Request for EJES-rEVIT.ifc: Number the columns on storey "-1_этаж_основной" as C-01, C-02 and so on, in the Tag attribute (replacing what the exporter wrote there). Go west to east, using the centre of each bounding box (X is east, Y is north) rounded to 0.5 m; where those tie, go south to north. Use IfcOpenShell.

First a look at what the model holds.

```python
import ifcopenshell
import ifcopenshell.util.element
import ifcopenshell.util.placement

model = ifcopenshell.open("EJES-rEVIT.ifc")
print(model.schema)
storey = next(s for s in model.by_type("IfcBuildingStorey") if s.Name == "-1_этаж_основной")
columns = [e for e in ifcopenshell.util.element.get_decomposition(storey) if e.is_a("IfcColumn")]
for e in sorted(columns, key=lambda e: e.id()):
    origin = ifcopenshell.util.placement.get_local_placement(e.ObjectPlacement)[:3, 3]
    print(e.id(), e.Tag, e.Name, origin.round(2) + 0.0, sep=" | ")
```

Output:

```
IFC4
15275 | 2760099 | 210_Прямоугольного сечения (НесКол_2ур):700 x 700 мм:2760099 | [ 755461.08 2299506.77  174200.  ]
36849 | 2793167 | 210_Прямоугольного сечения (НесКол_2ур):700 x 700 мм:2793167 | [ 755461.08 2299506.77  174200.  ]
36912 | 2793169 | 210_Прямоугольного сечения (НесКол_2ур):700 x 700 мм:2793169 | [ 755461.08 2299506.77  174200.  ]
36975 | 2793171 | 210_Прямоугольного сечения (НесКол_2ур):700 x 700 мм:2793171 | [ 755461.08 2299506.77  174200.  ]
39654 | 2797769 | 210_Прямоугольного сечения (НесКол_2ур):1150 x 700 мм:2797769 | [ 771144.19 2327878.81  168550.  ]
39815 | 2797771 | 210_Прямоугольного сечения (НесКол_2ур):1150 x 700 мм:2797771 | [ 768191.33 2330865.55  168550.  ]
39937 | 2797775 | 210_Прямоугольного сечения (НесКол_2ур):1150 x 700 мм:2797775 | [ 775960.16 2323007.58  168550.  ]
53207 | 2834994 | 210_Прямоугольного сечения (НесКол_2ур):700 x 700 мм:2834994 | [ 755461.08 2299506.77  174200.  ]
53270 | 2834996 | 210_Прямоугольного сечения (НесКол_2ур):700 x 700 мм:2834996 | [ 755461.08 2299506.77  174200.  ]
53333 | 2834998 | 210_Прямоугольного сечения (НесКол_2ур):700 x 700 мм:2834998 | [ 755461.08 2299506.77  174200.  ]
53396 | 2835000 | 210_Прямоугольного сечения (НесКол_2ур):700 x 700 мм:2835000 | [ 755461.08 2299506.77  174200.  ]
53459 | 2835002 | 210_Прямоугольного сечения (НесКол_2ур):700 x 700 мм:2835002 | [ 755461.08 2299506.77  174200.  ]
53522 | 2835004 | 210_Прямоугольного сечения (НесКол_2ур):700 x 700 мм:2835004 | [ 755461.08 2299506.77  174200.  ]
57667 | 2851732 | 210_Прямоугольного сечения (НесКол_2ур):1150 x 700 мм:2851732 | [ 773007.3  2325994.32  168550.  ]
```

```python
import ifcopenshell
import ifcopenshell.geom
import ifcopenshell.util.element
import ifcopenshell.util.shape

model = ifcopenshell.open("EJES-rEVIT.ifc")
settings = ifcopenshell.geom.settings()
settings.set("use-world-coords", True)


def centre(element):
    shape = ifcopenshell.geom.create_shape(settings, element)
    return ifcopenshell.util.shape.get_bbox_centroid(shape.geometry)


storey = next(s for s in model.by_type("IfcBuildingStorey") if s.Name == "-1_этаж_основной")
columns = [e for e in ifcopenshell.util.element.get_decomposition(storey) if e.is_a("IfcColumn")]

# Insertion points can sit at a corner or the storey origin, so sort by the geometry (in metres).
centres = {e: centre(e) for e in columns}
columns.sort(key=lambda e: (round(centres[e][0] / 0.5), centres[e][1]))

for i, e in enumerate(columns, start=1):
    number = f"C-{i:02d}"
    e.Tag = number
    print(e.id(), number)

model.write("EJES-rEVIT_edited.ifc")
```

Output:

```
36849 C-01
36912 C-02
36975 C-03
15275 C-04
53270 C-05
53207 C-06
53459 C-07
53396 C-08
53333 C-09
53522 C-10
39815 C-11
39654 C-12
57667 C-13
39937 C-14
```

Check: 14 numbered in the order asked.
